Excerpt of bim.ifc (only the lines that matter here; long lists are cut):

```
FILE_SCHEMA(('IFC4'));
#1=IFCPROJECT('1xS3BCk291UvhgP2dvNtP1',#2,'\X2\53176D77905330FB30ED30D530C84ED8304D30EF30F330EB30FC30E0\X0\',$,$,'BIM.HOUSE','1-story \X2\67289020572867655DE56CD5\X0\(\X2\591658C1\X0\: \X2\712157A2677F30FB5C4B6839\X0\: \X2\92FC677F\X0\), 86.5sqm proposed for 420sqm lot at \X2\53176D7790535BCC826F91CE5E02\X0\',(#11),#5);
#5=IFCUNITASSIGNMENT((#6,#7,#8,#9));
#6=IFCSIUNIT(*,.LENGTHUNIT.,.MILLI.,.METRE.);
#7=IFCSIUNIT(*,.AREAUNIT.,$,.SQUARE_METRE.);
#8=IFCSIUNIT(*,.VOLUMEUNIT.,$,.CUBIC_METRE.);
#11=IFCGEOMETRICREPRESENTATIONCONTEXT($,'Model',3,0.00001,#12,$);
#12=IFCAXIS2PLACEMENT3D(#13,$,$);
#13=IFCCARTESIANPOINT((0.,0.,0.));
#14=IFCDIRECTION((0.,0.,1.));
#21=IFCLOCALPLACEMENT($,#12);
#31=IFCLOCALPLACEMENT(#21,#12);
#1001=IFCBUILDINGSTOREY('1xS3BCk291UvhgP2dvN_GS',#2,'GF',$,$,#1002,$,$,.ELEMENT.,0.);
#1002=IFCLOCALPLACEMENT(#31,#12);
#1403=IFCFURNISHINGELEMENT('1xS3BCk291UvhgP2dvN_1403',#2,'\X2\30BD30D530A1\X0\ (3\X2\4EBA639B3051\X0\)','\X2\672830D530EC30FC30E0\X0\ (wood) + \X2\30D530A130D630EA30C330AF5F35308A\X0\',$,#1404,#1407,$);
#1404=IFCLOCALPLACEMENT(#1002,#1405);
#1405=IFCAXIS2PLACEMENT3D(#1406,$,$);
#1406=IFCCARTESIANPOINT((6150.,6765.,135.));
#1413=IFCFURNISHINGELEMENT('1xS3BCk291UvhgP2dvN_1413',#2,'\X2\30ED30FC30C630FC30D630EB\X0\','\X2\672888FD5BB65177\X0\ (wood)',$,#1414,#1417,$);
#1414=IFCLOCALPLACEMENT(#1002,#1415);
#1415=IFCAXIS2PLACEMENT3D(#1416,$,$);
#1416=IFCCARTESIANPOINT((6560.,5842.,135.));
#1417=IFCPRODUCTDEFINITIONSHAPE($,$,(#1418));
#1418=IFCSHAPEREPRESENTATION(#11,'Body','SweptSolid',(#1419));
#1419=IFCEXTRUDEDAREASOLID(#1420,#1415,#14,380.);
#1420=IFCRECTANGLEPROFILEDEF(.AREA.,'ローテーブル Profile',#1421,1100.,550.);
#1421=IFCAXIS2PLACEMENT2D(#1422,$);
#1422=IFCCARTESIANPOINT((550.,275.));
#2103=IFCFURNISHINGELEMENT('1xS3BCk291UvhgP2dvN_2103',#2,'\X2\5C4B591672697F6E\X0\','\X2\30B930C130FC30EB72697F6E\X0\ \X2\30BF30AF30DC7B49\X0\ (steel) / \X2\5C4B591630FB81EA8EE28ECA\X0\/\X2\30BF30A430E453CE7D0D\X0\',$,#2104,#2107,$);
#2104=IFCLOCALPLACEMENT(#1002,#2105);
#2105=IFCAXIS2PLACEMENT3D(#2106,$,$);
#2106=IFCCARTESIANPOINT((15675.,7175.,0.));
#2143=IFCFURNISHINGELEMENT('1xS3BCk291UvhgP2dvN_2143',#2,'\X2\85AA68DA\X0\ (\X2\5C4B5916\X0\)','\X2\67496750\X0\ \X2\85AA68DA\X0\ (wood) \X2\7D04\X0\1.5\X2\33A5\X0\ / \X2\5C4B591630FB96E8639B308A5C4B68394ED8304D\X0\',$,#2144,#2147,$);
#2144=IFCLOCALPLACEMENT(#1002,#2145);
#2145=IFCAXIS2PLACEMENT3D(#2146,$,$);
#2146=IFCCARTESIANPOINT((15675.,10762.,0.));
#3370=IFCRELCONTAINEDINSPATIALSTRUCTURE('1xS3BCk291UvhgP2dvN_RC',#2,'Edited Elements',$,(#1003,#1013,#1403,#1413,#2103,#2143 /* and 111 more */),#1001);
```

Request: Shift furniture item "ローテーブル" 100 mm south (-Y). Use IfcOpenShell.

```python
import ifcopenshell
import ifcopenshell.api.geometry
import ifcopenshell.util.placement
import ifcopenshell.util.unit

model = ifcopenshell.open("bim.ifc")
unit_scale = ifcopenshell.util.unit.calculate_unit_scale(model)

item = model.by_guid("1xS3BCk291UvhgP2dvN_1413")
matrix = ifcopenshell.util.placement.get_local_placement(item.ObjectPlacement)
matrix[1, 3] -= 0.1 / unit_scale
ifcopenshell.api.geometry.edit_object_placement(model, product=item, matrix=matrix, is_si=False)

print(ifcopenshell.util.placement.get_local_placement(item.ObjectPlacement).round(3) + 0.0)

model.write("bim_edited.ifc")
```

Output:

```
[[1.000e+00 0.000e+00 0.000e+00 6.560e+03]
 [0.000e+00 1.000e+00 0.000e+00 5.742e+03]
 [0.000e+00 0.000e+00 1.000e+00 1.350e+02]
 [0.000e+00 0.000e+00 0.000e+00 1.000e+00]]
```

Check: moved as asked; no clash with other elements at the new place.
